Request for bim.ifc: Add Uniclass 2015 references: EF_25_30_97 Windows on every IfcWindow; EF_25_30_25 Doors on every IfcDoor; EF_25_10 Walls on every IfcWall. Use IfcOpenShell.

First a look at what the model holds.

```python
import ifcopenshell

model = ifcopenshell.open("bim.ifc")
print(model.schema)
print("classifications:", [c.Name for c in model.by_type("IfcClassification")])
for ifc_class in ("IfcDoor", "IfcRoof", "IfcStair", "IfcWall", "IfcWindow"):
    print(ifc_class, len(model.by_type(ifc_class)))
```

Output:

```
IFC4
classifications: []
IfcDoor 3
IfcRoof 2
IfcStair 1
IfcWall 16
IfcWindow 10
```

```python
import ifcopenshell
import ifcopenshell.api.classification

model = ifcopenshell.open("bim.ifc")

system = ifcopenshell.api.classification.add_classification(model, classification="Uniclass 2015")

codes = {
    "IfcWindow": ("EF_25_30_97", "Windows"),
    "IfcDoor": ("EF_25_30_25", "Doors"),
    "IfcWall": ("EF_25_10", "Walls"),
}
for ifc_class, (code, name) in codes.items():
    products = model.by_type(ifc_class)
    ifcopenshell.api.classification.add_reference(
        model, products=products, classification=system, identification=code, name=name
    )
    print(code, len(products))

model.write("bim_v2.ifc")
```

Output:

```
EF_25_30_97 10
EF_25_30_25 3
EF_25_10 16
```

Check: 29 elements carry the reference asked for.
